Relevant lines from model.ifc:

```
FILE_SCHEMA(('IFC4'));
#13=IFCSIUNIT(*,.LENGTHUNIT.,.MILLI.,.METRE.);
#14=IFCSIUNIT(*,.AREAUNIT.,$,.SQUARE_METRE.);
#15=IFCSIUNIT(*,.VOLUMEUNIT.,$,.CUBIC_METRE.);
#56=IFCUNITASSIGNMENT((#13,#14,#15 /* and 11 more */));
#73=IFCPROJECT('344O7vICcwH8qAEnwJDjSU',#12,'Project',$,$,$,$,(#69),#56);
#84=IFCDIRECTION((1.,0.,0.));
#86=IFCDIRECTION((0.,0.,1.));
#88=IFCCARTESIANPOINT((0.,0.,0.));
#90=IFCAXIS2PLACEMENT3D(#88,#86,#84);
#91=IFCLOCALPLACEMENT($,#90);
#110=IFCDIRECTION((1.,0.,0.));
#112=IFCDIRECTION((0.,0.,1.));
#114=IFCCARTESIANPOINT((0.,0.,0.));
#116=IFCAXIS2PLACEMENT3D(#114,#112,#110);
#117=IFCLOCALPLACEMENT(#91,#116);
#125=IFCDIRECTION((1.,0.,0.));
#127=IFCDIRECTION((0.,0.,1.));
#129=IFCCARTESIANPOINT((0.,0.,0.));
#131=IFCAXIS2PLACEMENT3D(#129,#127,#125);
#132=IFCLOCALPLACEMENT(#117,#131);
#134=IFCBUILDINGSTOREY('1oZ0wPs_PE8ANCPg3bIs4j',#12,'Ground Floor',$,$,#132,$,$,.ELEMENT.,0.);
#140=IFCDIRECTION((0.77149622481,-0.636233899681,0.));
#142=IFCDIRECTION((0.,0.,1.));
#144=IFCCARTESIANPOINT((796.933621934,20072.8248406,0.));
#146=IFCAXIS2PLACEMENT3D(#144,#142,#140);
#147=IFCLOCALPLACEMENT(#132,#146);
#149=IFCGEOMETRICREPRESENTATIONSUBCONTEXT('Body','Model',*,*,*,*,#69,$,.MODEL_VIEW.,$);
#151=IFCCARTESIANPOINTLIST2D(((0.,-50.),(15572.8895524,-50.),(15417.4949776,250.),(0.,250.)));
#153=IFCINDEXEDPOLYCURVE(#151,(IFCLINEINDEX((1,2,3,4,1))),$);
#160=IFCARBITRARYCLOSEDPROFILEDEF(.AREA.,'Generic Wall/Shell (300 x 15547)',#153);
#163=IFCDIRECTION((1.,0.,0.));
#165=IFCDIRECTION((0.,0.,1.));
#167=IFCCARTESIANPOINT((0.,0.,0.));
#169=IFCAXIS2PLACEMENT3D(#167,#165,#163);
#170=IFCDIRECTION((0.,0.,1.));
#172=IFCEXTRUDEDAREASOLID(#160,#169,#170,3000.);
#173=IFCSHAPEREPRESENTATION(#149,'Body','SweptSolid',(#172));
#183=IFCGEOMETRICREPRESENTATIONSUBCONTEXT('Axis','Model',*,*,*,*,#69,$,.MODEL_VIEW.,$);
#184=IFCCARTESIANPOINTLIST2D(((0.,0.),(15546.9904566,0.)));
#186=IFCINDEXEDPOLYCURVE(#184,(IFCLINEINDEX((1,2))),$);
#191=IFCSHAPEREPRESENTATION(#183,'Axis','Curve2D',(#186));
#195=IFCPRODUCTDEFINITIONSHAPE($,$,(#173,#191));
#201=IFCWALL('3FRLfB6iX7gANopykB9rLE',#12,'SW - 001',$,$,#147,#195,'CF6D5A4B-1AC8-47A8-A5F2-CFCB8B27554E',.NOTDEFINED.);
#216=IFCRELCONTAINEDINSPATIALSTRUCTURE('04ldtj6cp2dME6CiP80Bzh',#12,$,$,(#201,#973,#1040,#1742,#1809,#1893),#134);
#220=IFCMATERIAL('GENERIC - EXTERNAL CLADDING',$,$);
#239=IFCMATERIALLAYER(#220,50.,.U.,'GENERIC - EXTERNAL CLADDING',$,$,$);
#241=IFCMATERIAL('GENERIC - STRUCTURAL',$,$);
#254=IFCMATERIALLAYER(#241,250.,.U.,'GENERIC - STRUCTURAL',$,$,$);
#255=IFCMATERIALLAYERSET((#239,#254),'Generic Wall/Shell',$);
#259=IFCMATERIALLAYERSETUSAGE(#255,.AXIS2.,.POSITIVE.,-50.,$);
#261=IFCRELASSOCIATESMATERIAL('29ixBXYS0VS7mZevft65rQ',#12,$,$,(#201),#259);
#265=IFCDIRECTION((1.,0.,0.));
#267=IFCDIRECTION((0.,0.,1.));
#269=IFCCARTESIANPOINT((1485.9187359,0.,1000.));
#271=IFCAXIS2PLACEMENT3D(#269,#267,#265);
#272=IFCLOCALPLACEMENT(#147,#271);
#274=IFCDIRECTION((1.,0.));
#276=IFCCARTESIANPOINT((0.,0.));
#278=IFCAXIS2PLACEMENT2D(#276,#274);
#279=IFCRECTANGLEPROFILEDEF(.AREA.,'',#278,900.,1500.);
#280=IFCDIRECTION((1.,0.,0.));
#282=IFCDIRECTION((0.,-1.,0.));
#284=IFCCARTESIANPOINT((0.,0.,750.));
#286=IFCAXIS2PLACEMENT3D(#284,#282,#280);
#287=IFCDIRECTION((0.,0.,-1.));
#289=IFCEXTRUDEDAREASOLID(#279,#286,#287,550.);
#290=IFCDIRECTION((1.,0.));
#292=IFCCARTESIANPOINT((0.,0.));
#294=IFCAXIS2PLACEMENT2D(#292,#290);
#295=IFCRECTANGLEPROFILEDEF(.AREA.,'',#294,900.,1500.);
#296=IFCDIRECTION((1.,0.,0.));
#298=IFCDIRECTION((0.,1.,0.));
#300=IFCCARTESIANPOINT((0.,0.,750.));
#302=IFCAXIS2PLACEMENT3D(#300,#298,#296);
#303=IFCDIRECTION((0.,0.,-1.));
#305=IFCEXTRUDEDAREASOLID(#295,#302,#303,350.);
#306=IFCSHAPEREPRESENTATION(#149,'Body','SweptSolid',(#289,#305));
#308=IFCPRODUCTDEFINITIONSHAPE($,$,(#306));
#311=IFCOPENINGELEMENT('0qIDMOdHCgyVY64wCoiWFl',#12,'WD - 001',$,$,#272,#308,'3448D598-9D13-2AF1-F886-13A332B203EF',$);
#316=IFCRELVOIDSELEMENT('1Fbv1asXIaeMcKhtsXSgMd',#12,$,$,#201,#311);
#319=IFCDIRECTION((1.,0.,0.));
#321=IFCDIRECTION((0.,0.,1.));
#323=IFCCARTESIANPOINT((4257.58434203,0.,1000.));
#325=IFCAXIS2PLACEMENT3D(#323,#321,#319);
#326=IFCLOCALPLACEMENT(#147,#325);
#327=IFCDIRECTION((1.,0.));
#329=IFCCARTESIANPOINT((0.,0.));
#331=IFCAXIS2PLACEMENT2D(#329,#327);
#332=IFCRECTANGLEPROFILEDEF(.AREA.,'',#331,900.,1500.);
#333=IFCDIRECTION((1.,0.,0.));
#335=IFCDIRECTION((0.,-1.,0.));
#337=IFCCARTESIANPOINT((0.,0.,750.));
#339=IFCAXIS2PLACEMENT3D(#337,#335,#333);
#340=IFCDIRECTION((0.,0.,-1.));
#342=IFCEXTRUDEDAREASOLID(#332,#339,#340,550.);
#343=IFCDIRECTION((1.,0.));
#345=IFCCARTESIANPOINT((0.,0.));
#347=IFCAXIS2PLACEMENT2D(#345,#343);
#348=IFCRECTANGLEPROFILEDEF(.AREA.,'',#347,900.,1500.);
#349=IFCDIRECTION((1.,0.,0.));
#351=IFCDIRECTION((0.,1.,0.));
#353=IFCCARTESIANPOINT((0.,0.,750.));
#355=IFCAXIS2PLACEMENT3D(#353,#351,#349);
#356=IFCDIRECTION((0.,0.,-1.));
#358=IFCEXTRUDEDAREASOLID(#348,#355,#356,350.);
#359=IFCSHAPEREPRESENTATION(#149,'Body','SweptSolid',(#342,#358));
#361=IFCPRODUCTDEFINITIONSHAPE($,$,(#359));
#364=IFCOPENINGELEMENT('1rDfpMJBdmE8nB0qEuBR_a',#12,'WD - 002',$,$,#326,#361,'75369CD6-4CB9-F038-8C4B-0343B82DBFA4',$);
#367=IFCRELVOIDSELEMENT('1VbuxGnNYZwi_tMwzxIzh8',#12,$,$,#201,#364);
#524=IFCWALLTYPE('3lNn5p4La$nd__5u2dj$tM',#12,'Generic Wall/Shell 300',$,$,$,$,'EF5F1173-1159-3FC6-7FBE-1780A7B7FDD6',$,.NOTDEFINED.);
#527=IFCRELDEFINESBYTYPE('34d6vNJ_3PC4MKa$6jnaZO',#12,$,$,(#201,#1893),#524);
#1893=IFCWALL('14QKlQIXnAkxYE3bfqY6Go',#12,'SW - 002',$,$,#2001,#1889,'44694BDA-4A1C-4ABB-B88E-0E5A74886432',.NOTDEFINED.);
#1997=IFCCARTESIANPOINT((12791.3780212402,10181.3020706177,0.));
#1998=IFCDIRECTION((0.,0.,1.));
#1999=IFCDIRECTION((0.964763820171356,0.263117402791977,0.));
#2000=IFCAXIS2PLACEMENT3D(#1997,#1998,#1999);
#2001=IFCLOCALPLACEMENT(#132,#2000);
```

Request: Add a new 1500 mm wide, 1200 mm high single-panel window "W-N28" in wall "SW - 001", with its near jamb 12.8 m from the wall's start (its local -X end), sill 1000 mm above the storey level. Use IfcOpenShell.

```python
import numpy as np
import ifcopenshell
import ifcopenshell.api.feature
import ifcopenshell.api.geometry
import ifcopenshell.api.root
import ifcopenshell.api.spatial
import ifcopenshell.geom
import ifcopenshell.util.element
import ifcopenshell.util.placement
import ifcopenshell.util.representation
import ifcopenshell.util.shape
import ifcopenshell.util.unit

model = ifcopenshell.open("model.ifc")
unit_scale = ifcopenshell.util.unit.calculate_unit_scale(model)
settings = ifcopenshell.geom.settings()


def volume(element):
    """Net volume in cubic metres, openings subtracted."""
    shape = ifcopenshell.geom.create_shape(settings, element)
    return ifcopenshell.util.shape.get_volume(shape.geometry)


wall = model.by_guid("3FRLfB6iX7gANopykB9rLE")
storey = ifcopenshell.util.element.get_container(wall, ifc_class="IfcBuildingStorey")
context = ifcopenshell.util.representation.get_context(model, "Model", "Body", "MODEL_VIEW")
before = volume(wall)

width, height, from_end, sill = 1.5, 1.2, 12.8, 1  # metres

# The wall runs along its own X axis, and the end named is its -X end.
wall_shape = ifcopenshell.geom.create_shape(settings, wall)
x, y, z = ifcopenshell.util.shape.get_vertices(wall_shape.geometry).T
start = x.min() + from_end
face, thickness = float(y.min()), float(y.max() - y.min())
wall_matrix = ifcopenshell.util.placement.get_local_placement(wall.ObjectPlacement)
level = ifcopenshell.util.placement.get_local_placement(storey.ObjectPlacement)[2, 3]


def in_wall(x, y):
    """Placement at x, y metres in the wall's axes, at sill height."""
    matrix = wall_matrix.copy()
    matrix[:, 3] = wall_matrix @ np.array([x / unit_scale, y / unit_scale, 0.0, 1.0])
    matrix[2, 3] = level + sill / unit_scale
    return matrix


# Opening: a box that overshoots both wall faces by 50 mm.
opening = ifcopenshell.api.root.create_entity(model, ifc_class="IfcOpeningElement", predefined_type="OPENING")
box = ifcopenshell.api.geometry.add_wall_representation(
    model, context=context, length=width, height=height, thickness=thickness + 0.1
)
ifcopenshell.api.geometry.assign_representation(model, product=opening, representation=box)
ifcopenshell.api.geometry.edit_object_placement(model, product=opening, matrix=in_wall(start, face - 0.05), is_si=False)
ifcopenshell.api.feature.add_feature(model, feature=opening, element=wall)

window = ifcopenshell.api.root.create_entity(model, ifc_class="IfcWindow", name="W-N28", predefined_type="WINDOW")
window.OverallWidth, window.OverallHeight = width / unit_scale, height / unit_scale
window.PartitioningType = "SINGLE_PANEL"
body = ifcopenshell.api.geometry.add_window_representation(
    model,
    context=context,
    overall_width=window.OverallWidth,
    overall_height=window.OverallHeight,
    partition_type="SINGLE_PANEL",
)
ifcopenshell.api.geometry.assign_representation(model, product=window, representation=body)
ifcopenshell.api.spatial.assign_container(model, products=[window], relating_structure=storey)
ifcopenshell.api.feature.add_filling(model, opening=opening, element=window)

# Centre the window in the wall's thickness.
ifcopenshell.api.geometry.edit_object_placement(model, product=window, matrix=in_wall(start, face), is_si=False)
window_shape = ifcopenshell.geom.create_shape(settings, window)
depth = ifcopenshell.util.shape.get_vertices(window_shape.geometry)[:, 1]
offset = face + thickness / 2 - (depth.min() + depth.max()) / 2
ifcopenshell.api.geometry.edit_object_placement(model, product=window, matrix=in_wall(start, offset), is_si=False)

after = volume(wall)

print(f"wall volume {before:.3f} -> {after:.3f} m3")

model.write("model-out.ifc")
```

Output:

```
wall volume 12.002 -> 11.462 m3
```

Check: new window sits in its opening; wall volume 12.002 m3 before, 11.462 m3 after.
